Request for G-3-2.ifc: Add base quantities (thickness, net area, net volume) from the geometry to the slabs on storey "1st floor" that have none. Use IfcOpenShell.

First a look at what the model holds.

```python
import ifcopenshell
import ifcopenshell.util.element
import ifcopenshell.util.unit

model = ifcopenshell.open("G-3-2.ifc")
print(model.schema)
for unit_type in ("LENGTHUNIT", "AREAUNIT", "VOLUMEUNIT"):
    print(unit_type, ifcopenshell.util.unit.calculate_unit_scale(model, unit_type))
storey = next(s for s in model.by_type("IfcBuildingStorey") if s.Name == "1st floor")
slabs = [e for e in ifcopenshell.util.element.get_decomposition(storey) if e.is_a("IfcSlab")]
for e in sorted(slabs, key=lambda e: e.id()):
    print(e.id(), e.is_a(), e.Name, list(ifcopenshell.util.element.get_psets(e, qtos_only=True)), sep=" | ")
```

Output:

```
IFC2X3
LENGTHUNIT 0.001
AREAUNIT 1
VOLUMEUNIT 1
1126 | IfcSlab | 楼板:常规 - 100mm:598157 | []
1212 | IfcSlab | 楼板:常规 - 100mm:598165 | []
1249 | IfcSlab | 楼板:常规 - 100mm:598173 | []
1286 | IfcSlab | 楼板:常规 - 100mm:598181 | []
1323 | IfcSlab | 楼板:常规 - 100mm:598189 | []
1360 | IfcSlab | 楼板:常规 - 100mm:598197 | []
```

```python
import ifcopenshell
import ifcopenshell.api.pset
import ifcopenshell.geom
import ifcopenshell.util.element
import ifcopenshell.util.shape
import ifcopenshell.util.unit

model = ifcopenshell.open("G-3-2.ifc")
unit_scale = ifcopenshell.util.unit.calculate_unit_scale(model)
area_scale = ifcopenshell.util.unit.calculate_unit_scale(model, "AREAUNIT")
volume_scale = ifcopenshell.util.unit.calculate_unit_scale(model, "VOLUMEUNIT")
settings = ifcopenshell.geom.settings()

storey = next(s for s in model.by_type("IfcBuildingStorey") if s.Name == "1st floor")
slabs = [e for e in ifcopenshell.util.element.get_decomposition(storey) if e.is_a("IfcSlab")]

for e in sorted(slabs, key=lambda e: e.id()):
    if ifcopenshell.util.element.get_psets(e, qtos_only=True, should_inherit=False):
        continue
    # Geometry comes back in metres, in the element's own axes.
    shape = ifcopenshell.geom.create_shape(settings, e)
    values = {
        "Width": ifcopenshell.util.shape.get_z(shape.geometry) / unit_scale,
        "NetArea": ifcopenshell.util.shape.get_footprint_area(shape.geometry) / area_scale,
        "NetVolume": ifcopenshell.util.shape.get_volume(shape.geometry) / volume_scale,
    }
    qto = ifcopenshell.api.pset.add_qto(model, product=e, name="BaseQuantities")
    ifcopenshell.api.pset.edit_qto(model, qto=qto, properties=values)
    print(e.id(), {k: round(v, 3) for k, v in values.items()})

model.write("G-3-2_v2.ifc")
```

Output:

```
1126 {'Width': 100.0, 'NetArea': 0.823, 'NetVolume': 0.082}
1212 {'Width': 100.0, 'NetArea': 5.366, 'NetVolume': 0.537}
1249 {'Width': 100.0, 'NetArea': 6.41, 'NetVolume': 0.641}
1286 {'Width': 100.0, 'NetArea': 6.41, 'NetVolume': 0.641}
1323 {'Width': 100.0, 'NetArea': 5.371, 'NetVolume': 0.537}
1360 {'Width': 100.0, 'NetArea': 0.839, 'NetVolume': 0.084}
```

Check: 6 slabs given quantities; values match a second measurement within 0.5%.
